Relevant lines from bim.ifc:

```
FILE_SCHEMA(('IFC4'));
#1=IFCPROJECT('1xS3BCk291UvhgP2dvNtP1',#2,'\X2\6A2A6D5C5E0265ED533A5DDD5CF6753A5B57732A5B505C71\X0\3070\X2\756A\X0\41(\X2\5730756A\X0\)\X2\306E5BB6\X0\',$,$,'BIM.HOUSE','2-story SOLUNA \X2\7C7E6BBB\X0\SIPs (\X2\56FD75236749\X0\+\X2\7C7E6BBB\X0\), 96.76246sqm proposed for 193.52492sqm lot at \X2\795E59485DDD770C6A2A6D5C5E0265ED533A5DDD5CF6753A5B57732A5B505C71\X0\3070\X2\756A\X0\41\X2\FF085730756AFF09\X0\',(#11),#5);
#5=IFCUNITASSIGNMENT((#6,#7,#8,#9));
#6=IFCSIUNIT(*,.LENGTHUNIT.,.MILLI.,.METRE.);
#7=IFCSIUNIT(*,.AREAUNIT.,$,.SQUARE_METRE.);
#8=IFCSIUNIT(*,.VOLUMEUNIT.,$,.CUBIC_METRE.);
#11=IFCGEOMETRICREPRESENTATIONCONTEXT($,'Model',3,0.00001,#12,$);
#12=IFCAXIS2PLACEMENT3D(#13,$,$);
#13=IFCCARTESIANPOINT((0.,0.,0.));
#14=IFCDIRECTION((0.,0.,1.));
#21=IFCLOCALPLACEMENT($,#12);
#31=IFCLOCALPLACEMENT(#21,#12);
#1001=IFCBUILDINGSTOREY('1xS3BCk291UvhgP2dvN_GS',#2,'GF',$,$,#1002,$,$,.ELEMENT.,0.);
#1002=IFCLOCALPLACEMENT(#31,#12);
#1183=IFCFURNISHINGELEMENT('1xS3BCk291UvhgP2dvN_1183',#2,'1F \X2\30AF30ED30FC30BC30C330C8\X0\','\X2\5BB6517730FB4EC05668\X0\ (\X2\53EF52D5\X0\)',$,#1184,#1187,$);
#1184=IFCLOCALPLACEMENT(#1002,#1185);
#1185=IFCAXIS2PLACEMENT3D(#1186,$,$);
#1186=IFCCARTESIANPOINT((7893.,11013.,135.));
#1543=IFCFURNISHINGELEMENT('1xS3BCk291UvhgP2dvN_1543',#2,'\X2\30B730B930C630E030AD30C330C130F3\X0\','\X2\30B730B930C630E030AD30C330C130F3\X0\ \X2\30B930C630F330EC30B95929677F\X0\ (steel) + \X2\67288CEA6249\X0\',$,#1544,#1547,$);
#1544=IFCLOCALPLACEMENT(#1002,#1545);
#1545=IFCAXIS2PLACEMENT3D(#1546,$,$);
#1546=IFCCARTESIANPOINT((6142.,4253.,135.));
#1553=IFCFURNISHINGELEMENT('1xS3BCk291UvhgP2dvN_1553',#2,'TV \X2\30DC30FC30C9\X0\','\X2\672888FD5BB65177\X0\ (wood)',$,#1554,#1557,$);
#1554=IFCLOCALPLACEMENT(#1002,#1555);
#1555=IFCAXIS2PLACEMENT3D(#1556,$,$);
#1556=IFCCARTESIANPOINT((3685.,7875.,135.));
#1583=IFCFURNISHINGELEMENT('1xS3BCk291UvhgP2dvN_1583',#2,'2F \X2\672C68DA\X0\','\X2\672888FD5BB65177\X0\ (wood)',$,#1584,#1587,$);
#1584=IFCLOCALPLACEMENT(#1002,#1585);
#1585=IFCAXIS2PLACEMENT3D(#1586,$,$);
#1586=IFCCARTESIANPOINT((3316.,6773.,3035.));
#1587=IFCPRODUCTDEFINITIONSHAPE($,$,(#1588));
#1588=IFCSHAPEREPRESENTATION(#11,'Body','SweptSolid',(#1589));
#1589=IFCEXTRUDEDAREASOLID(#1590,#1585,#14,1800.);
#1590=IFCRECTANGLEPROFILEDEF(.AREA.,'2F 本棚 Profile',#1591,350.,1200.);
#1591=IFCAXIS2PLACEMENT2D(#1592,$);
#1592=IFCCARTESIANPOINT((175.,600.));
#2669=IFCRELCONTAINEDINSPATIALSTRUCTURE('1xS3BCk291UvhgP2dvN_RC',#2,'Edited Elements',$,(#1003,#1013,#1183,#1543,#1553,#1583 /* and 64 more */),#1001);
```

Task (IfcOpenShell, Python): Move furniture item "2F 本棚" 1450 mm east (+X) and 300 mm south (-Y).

```python
import ifcopenshell
import ifcopenshell.api.geometry
import ifcopenshell.util.placement
import ifcopenshell.util.unit

model = ifcopenshell.open("bim.ifc")
unit_scale = ifcopenshell.util.unit.calculate_unit_scale(model)

item = model.by_guid("1xS3BCk291UvhgP2dvN_1583")
matrix = ifcopenshell.util.placement.get_local_placement(item.ObjectPlacement)
matrix[0, 3] += 1.45 / unit_scale
matrix[1, 3] -= 0.3 / unit_scale
ifcopenshell.api.geometry.edit_object_placement(model, product=item, matrix=matrix, is_si=False)

print(ifcopenshell.util.placement.get_local_placement(item.ObjectPlacement).round(3) + 0.0)

model.write("bim_rev.ifc")
```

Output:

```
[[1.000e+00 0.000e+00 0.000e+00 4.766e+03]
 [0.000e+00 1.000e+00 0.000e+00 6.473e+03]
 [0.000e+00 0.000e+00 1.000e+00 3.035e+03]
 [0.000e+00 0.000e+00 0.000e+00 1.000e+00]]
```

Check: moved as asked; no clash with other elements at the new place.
